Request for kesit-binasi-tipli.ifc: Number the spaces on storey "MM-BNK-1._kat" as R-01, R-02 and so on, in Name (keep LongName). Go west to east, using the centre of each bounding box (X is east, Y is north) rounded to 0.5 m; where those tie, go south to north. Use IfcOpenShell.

First a look at what the model holds.

```python
import ifcopenshell
import ifcopenshell.util.element
import ifcopenshell.util.placement

model = ifcopenshell.open("kesit-binasi-tipli.ifc")
print(model.schema)
storey = next(s for s in model.by_type("IfcBuildingStorey") if s.Name == "MM-BNK-1._kat")
spaces = [e for e in ifcopenshell.util.element.get_decomposition(storey) if e.is_a("IfcSpace")]
for e in sorted(spaces, key=lambda e: e.id()):
    origin = ifcopenshell.util.placement.get_local_placement(e.ObjectPlacement)[:3, 3]
    print(e.id(), e.Name, e.LongName, origin.round(2) + 0.0, sep=" | ")
```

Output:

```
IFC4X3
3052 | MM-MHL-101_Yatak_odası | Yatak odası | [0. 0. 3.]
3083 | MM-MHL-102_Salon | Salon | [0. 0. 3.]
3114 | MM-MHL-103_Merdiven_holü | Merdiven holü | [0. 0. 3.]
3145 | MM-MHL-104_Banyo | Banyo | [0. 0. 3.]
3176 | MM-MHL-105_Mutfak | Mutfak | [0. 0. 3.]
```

```python
import ifcopenshell
import ifcopenshell.geom
import ifcopenshell.util.element
import ifcopenshell.util.shape

model = ifcopenshell.open("kesit-binasi-tipli.ifc")
settings = ifcopenshell.geom.settings()
settings.set("use-world-coords", True)


def centre(element):
    shape = ifcopenshell.geom.create_shape(settings, element)
    return ifcopenshell.util.shape.get_bbox_centroid(shape.geometry)


storey = next(s for s in model.by_type("IfcBuildingStorey") if s.Name == "MM-BNK-1._kat")
spaces = [e for e in ifcopenshell.util.element.get_decomposition(storey) if e.is_a("IfcSpace")]

# Insertion points can sit at a corner or the storey origin, so sort by the geometry (in metres).
centres = {e: centre(e) for e in spaces}
spaces.sort(key=lambda e: (round(centres[e][0] / 0.5), centres[e][1]))

for i, e in enumerate(spaces, start=1):
    number = f"R-{i:02d}"
    e.Name = number
    print(e.id(), number)

model.write("kesit-binasi-tipli_updated.ifc")
```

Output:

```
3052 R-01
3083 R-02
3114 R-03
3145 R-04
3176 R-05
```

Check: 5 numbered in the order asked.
